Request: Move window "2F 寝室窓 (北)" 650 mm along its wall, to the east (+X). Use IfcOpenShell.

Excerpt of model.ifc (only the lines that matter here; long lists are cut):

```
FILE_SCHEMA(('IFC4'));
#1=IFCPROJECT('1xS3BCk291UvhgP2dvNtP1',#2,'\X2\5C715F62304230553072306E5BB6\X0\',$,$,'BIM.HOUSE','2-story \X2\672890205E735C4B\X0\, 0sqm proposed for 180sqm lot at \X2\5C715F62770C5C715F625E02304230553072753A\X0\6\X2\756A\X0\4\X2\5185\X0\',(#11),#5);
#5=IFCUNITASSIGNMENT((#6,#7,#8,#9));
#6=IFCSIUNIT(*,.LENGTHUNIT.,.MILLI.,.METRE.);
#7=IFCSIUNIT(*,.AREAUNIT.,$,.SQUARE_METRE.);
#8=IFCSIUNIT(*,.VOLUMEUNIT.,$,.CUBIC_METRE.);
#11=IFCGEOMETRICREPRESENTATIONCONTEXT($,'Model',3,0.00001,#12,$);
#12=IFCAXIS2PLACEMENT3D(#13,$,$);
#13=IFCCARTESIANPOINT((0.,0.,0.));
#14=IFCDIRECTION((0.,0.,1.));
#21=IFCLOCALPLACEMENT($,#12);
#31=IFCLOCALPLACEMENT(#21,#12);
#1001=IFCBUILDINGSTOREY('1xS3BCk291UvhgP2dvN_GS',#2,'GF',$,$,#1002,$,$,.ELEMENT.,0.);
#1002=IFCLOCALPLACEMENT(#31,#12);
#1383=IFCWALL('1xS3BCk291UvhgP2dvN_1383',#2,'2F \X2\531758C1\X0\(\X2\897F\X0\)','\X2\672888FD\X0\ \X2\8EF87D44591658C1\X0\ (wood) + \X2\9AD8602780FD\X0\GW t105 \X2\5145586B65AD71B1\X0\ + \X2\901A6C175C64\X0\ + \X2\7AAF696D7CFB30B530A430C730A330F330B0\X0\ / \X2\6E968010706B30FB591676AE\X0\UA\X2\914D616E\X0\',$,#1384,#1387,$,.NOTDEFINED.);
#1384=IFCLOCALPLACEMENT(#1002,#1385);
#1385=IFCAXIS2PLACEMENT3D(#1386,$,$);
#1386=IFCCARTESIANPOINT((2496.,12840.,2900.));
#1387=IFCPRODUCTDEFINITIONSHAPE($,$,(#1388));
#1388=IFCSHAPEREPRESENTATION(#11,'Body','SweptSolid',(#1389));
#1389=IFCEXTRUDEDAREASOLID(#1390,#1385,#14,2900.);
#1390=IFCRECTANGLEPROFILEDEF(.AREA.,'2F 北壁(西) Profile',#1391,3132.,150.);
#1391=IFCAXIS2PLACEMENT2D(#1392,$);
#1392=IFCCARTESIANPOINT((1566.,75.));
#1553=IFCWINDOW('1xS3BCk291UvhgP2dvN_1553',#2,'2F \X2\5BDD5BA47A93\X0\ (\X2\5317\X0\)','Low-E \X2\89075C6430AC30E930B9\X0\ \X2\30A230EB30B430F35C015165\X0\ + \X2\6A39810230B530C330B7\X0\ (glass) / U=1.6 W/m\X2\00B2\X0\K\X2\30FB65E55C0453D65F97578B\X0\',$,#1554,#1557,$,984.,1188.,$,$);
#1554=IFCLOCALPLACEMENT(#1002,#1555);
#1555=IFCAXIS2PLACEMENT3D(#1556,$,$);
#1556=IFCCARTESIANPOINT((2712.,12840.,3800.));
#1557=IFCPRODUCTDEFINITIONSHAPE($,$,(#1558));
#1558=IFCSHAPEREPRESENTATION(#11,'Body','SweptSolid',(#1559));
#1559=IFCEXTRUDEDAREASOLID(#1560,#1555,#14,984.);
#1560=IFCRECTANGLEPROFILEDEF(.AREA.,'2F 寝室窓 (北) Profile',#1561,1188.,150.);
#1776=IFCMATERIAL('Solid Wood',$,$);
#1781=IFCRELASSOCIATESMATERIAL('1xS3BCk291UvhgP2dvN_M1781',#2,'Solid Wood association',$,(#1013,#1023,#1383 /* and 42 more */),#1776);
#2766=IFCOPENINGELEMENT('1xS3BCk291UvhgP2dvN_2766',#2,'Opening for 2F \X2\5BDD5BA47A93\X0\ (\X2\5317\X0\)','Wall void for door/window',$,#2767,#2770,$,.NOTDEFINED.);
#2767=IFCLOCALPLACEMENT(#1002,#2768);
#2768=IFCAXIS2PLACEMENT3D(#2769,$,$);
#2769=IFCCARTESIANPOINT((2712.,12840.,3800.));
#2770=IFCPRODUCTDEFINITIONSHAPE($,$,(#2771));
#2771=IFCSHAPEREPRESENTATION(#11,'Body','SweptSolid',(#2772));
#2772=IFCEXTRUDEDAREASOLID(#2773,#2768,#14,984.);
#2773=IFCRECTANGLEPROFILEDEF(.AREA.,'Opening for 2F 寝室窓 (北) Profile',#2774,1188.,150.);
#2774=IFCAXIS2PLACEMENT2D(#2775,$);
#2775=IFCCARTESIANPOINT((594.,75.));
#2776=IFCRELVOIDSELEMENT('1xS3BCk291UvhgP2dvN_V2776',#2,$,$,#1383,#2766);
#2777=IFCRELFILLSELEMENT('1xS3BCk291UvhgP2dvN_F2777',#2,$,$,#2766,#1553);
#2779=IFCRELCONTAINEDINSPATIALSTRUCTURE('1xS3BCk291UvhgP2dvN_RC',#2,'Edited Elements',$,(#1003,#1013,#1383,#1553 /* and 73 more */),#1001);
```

```python
import ifcopenshell
import ifcopenshell.api.geometry
import ifcopenshell.util.placement

model = ifcopenshell.open("model.ifc")

window = model.by_guid("1xS3BCk291UvhgP2dvN_1553")
opening = window.FillsVoids[0].RelatingOpeningElement
wall = opening.VoidsElements[0].RelatingBuildingElement

wall_matrix = ifcopenshell.util.placement.get_local_placement(wall.ObjectPlacement)
shift = wall_matrix[:3, 0] * 650.0
before = ifcopenshell.util.placement.get_local_placement(window.ObjectPlacement)[:3, 3].copy()

# The window is not placed relative to its opening, so move both.
for product in (opening, window):
    matrix = ifcopenshell.util.placement.get_local_placement(product.ObjectPlacement)
    matrix[:3, 3] += shift
    ifcopenshell.api.geometry.edit_object_placement(model, product=product, matrix=matrix, is_si=False)

after = ifcopenshell.util.placement.get_local_placement(window.ObjectPlacement)[:3, 3]
print("window moved by", (after - before).round(3) + 0.0)

model.write("model_v2.ifc")
```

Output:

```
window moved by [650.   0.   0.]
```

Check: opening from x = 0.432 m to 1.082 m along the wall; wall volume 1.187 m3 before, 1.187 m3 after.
